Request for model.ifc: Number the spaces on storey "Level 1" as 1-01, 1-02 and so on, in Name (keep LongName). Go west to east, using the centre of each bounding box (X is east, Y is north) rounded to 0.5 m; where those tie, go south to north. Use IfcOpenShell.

First a look at what the model holds.

```python
import ifcopenshell
import ifcopenshell.util.element
import ifcopenshell.util.placement

model = ifcopenshell.open("model.ifc")
print(model.schema)
storey = next(s for s in model.by_type("IfcBuildingStorey") if s.Name == "Level 1")
spaces = [e for e in ifcopenshell.util.element.get_decomposition(storey) if e.is_a("IfcSpace")]
for e in sorted(spaces, key=lambda e: e.id()):
    origin = ifcopenshell.util.placement.get_local_placement(e.ObjectPlacement)[:3, 3]
    print(e.id(), e.Name, e.LongName, origin.round(2) + 0.0, sep=" | ")
```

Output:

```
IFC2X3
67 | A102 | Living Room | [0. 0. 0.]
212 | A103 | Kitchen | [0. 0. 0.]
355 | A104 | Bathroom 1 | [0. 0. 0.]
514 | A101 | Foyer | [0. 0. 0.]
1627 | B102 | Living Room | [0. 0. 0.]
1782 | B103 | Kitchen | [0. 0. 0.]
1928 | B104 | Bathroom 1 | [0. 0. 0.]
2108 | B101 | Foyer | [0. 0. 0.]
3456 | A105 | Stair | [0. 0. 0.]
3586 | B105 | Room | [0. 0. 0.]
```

```python
import ifcopenshell
import ifcopenshell.geom
import ifcopenshell.util.element
import ifcopenshell.util.shape

model = ifcopenshell.open("model.ifc")
settings = ifcopenshell.geom.settings()
settings.set("use-world-coords", True)


def centre(element):
    shape = ifcopenshell.geom.create_shape(settings, element)
    return ifcopenshell.util.shape.get_bbox_centroid(shape.geometry)


storey = next(s for s in model.by_type("IfcBuildingStorey") if s.Name == "Level 1")
spaces = [e for e in ifcopenshell.util.element.get_decomposition(storey) if e.is_a("IfcSpace")]

# Insertion points can sit at a corner or the storey origin, so sort by the geometry (in metres).
centres = {e: centre(e) for e in spaces}
spaces.sort(key=lambda e: (round(centres[e][0] / 0.5), centres[e][1]))

for i, e in enumerate(spaces, start=1):
    number = f"1-{i:02d}"
    e.Name = number
    print(e.id(), number)

model.write("model_v2.ifc")
```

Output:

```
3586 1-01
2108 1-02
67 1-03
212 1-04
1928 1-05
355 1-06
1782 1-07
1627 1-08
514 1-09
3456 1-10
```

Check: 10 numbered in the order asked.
